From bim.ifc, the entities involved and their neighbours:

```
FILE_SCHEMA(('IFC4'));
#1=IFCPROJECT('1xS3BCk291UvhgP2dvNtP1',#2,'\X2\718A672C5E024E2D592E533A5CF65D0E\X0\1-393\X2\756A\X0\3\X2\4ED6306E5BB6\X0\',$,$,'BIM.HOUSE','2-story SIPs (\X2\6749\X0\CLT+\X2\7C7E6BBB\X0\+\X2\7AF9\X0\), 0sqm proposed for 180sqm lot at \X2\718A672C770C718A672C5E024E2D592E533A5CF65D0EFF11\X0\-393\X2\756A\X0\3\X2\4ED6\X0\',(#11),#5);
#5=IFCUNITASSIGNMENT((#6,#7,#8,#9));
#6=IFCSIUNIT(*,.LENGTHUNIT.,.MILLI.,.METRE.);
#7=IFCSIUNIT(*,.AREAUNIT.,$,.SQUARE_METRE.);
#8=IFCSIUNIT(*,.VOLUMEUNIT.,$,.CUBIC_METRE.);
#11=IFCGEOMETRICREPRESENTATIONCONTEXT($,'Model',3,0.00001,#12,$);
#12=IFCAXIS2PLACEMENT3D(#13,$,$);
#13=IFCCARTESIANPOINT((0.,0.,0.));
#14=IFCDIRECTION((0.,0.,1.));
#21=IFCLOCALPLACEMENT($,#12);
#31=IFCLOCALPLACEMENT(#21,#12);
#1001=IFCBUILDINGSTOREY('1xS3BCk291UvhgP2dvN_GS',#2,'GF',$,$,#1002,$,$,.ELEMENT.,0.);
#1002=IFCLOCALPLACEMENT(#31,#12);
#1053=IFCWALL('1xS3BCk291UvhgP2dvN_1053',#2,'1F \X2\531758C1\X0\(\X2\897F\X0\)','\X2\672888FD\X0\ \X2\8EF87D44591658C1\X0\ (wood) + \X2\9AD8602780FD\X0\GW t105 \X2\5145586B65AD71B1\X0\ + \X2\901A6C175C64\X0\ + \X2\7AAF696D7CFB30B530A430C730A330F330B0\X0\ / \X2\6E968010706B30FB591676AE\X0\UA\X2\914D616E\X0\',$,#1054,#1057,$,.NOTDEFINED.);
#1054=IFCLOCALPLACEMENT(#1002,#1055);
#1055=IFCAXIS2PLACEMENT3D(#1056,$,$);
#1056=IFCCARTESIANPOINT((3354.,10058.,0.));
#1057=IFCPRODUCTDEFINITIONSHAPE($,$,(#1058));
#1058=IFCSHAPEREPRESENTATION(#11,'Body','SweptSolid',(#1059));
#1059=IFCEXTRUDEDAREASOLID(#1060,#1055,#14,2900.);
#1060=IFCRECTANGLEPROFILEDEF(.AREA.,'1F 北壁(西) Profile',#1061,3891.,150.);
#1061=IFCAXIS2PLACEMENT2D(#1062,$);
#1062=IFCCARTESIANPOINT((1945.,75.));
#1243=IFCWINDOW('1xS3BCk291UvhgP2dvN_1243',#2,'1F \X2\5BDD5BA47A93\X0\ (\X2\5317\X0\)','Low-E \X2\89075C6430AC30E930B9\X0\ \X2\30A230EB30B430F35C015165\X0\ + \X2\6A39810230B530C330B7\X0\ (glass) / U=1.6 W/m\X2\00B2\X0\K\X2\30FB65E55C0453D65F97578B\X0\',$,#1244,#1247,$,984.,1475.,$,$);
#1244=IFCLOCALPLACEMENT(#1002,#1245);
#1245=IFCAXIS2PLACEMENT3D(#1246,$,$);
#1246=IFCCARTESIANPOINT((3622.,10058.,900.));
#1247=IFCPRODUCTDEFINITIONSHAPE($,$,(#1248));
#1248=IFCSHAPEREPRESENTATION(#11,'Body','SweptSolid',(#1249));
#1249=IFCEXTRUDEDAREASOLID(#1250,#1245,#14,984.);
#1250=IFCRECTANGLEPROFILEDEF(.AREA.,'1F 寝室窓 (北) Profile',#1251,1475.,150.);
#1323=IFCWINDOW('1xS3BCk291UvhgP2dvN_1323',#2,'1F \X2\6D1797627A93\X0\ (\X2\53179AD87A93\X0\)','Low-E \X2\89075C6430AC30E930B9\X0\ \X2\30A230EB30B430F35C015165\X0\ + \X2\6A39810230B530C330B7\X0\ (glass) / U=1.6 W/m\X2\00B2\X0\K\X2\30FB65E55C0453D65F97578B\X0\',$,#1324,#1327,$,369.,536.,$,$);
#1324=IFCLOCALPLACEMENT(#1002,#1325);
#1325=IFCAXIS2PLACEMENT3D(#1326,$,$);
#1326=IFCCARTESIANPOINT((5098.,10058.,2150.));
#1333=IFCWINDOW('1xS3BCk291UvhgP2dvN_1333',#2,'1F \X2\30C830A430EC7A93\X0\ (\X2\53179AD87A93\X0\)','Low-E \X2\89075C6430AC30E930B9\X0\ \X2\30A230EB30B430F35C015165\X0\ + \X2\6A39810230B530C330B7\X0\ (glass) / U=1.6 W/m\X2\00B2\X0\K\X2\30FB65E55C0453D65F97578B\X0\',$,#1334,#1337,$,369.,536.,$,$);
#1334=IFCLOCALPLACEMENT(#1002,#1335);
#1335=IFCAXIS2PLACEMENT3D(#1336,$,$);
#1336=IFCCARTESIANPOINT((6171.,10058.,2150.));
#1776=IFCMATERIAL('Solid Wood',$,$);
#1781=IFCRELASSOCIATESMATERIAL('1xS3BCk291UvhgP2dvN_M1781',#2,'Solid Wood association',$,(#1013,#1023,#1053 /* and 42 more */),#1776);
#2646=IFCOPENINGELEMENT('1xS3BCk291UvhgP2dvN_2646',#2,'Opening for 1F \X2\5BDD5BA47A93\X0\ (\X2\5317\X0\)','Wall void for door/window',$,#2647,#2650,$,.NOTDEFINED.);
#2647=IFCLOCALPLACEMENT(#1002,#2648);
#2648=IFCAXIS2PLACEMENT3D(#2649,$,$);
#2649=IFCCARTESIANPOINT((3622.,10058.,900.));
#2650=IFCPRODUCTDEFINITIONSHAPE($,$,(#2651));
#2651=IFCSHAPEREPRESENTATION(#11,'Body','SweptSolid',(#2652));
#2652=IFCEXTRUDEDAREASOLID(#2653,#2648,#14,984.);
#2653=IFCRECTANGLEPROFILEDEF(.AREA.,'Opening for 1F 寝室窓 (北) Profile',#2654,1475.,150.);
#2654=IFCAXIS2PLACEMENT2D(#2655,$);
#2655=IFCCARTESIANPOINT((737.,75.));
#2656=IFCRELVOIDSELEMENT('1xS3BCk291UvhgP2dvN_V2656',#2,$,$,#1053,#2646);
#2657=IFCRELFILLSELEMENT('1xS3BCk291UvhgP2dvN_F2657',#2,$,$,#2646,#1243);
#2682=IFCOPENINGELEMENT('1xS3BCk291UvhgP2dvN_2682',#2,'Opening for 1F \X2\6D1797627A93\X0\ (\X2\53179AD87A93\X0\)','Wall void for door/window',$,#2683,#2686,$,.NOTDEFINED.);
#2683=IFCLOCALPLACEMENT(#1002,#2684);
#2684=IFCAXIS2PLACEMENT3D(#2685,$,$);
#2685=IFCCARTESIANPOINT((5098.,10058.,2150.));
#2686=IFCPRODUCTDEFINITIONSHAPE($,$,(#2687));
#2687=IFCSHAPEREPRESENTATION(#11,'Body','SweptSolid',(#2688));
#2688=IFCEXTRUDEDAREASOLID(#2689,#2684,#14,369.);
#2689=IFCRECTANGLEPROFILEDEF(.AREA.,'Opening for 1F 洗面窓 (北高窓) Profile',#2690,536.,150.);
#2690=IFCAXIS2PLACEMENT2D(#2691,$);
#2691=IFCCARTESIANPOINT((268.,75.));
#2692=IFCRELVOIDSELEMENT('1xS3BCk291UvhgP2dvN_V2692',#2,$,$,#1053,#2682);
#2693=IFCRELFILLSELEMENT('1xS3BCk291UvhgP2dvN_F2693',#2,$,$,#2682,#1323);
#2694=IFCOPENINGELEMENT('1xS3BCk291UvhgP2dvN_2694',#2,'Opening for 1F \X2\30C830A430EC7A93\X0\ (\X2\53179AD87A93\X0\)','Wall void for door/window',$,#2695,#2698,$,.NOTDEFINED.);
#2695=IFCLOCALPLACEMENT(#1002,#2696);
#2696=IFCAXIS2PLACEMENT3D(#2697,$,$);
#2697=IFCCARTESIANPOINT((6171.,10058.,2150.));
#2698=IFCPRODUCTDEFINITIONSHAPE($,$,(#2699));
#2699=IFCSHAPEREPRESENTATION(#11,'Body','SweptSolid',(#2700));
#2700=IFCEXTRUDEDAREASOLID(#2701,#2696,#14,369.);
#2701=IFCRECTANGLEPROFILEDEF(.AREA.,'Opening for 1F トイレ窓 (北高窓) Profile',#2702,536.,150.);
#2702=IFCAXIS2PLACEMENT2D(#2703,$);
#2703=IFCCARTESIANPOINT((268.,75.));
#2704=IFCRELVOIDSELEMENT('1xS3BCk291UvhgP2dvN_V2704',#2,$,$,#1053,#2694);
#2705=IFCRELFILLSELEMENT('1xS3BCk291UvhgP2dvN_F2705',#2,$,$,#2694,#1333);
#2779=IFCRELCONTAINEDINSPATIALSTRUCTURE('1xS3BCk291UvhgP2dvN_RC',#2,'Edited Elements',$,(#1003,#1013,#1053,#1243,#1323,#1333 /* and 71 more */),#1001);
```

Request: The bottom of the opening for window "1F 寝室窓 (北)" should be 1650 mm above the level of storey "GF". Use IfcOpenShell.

```python
import numpy as np
import ifcopenshell
import ifcopenshell.api.geometry
import ifcopenshell.geom
import ifcopenshell.util.element
import ifcopenshell.util.placement
import ifcopenshell.util.shape
import ifcopenshell.util.unit

model = ifcopenshell.open("bim.ifc")
unit_scale = ifcopenshell.util.unit.calculate_unit_scale(model)

window = model.by_id(1243)
opening = window.FillsVoids[0].RelatingOpeningElement
storey = ifcopenshell.util.element.get_container(window, ifc_class="IfcBuildingStorey")
level = ifcopenshell.util.placement.get_local_placement(storey.ObjectPlacement)[2, 3]

# The opening's origin need not be at the sill, so measure its lowest point.
shape = ifcopenshell.geom.create_shape(ifcopenshell.geom.settings(), opening)
bottom = ifcopenshell.util.shape.get_shape_bottom_elevation(shape, shape.geometry) / unit_scale
dz = level + 1.65 / unit_scale - bottom

shift = np.array([0.0, 0.0, dz])
# The window is not placed relative to its opening, so move both.
for product in (opening, window):
    matrix = ifcopenshell.util.placement.get_local_placement(product.ObjectPlacement)
    matrix[:3, 3] += shift
    ifcopenshell.api.geometry.edit_object_placement(model, product=product, matrix=matrix, is_si=False)

print(f"moved by {dz * unit_scale:+.3f} m")

model.write("bim-out.ifc")
```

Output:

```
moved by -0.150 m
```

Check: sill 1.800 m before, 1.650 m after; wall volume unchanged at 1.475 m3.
